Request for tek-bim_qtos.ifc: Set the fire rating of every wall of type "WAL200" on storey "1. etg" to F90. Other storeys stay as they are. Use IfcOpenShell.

First a look at what the model holds.

```python
import ifcopenshell
import ifcopenshell.util.element

model = ifcopenshell.open("tek-bim_qtos.ifc")
print(model.schema)
storey = next(s for s in model.by_type("IfcBuildingStorey") if s.Name == "1. etg")
walls = [e for e in ifcopenshell.util.element.get_decomposition(storey) if e.is_a("IfcWall")]
seen = {}
for e in walls:
    element_type = ifcopenshell.util.element.get_type(e)
    key = (element_type.Name if element_type != e and element_type else None, ifcopenshell.util.element.get_pset(e, "Pset_WallCommon", "FireRating"))
    seen[key] = seen.get(key, 0) + 1
for (name, value), count in sorted(seen.items(), key=str):
    print(count, "x", name, "|", value)
```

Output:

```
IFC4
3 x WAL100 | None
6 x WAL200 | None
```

```python
import ifcopenshell
import ifcopenshell.api.pset
import ifcopenshell.util.element

model = ifcopenshell.open("tek-bim_qtos.ifc")

storey = next(s for s in model.by_type("IfcBuildingStorey") if s.Name == "1. etg")
walls = [e for e in ifcopenshell.util.element.get_decomposition(storey) if e.is_a("IfcWall")]

count = 0
for e in walls:
    element_type = ifcopenshell.util.element.get_type(e)
    if element_type in (None, e) or element_type.Name != "WAL200":
        continue
    # add_pset returns the element's existing set when there is one.
    pset = ifcopenshell.api.pset.add_pset(model, product=e, name="Pset_WallCommon")
    ifcopenshell.api.pset.edit_pset(model, pset=pset, properties={"FireRating": "F90"})
    count += 1

print(count, "walls updated")

model.write("tek-bim_qtos_edited.ifc")
```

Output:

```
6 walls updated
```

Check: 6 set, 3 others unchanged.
